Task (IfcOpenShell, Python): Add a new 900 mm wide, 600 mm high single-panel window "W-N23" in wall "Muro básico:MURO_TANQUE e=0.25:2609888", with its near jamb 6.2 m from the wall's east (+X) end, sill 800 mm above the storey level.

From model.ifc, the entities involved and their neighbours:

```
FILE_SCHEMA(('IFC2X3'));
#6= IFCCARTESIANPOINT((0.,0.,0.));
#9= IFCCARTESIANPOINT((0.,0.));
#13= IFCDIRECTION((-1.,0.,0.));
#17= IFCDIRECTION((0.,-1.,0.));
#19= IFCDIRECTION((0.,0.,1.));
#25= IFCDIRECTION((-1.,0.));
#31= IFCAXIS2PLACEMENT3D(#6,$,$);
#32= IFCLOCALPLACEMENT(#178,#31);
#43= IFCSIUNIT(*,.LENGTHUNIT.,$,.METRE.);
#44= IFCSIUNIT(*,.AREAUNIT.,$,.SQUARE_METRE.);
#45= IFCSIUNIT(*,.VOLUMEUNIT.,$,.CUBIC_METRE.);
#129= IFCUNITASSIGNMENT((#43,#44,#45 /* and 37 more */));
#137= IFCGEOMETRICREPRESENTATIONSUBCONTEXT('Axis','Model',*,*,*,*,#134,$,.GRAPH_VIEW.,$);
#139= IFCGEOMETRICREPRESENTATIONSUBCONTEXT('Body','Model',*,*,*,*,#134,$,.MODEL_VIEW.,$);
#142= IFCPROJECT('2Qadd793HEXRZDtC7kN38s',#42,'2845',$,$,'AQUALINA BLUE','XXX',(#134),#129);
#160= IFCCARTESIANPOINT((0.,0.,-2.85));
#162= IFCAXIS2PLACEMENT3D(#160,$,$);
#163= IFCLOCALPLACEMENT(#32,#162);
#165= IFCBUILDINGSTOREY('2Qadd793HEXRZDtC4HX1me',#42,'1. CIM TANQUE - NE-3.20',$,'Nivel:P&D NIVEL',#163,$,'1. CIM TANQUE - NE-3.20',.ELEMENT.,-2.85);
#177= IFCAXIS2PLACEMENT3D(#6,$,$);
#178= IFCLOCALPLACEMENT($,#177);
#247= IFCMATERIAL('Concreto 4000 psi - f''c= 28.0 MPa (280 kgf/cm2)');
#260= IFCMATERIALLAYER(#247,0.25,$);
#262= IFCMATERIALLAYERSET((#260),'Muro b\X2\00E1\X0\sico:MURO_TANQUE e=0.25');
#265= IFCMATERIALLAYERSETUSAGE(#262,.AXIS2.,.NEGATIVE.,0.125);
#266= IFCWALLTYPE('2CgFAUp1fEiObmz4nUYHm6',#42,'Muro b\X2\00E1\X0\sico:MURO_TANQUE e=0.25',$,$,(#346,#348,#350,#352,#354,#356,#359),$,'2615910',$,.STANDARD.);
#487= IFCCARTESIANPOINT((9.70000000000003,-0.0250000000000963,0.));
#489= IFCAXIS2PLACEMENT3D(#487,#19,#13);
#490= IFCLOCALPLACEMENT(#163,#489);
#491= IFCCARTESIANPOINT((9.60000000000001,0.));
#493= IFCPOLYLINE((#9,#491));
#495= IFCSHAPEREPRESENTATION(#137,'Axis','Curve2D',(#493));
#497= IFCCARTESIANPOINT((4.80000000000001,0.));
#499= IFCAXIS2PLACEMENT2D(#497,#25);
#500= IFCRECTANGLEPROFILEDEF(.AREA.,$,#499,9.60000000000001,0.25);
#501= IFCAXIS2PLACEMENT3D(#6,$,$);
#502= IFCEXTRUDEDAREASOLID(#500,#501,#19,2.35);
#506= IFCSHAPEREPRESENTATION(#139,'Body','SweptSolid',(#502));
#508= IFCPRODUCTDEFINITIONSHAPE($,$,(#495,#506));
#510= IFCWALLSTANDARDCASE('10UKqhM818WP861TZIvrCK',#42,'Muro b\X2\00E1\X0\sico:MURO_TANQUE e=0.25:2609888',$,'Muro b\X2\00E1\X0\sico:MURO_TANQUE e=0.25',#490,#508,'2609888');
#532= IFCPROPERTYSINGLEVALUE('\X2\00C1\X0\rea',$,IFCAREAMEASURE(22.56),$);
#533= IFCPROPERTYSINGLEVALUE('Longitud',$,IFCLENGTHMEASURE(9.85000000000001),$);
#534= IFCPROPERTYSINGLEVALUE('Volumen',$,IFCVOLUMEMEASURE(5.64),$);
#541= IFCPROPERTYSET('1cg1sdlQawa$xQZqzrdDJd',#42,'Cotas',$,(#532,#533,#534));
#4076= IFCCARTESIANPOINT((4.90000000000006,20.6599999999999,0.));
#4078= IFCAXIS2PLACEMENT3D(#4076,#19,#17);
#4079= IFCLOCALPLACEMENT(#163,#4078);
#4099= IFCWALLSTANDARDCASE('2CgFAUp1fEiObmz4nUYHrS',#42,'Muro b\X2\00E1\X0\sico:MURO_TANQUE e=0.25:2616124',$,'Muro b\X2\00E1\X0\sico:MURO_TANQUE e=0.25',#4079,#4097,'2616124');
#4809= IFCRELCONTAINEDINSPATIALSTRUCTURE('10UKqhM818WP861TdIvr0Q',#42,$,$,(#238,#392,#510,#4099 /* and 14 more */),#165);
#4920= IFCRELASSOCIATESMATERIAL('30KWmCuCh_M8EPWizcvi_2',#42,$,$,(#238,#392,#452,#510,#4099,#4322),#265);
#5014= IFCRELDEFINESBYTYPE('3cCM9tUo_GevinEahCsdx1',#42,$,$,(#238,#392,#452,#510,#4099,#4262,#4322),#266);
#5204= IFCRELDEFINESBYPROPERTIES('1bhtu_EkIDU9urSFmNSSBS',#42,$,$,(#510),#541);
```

```python
import numpy as np
import ifcopenshell
import ifcopenshell.api.feature
import ifcopenshell.api.geometry
import ifcopenshell.api.pset
import ifcopenshell.api.root
import ifcopenshell.api.spatial
import ifcopenshell.api.type
import ifcopenshell.geom
import ifcopenshell.util.element
import ifcopenshell.util.placement
import ifcopenshell.util.representation
import ifcopenshell.util.shape
import ifcopenshell.util.unit

model = ifcopenshell.open("model.ifc")
unit_scale = ifcopenshell.util.unit.calculate_unit_scale(model)
area_scale = ifcopenshell.util.unit.calculate_unit_scale(model, "AREAUNIT")
volume_scale = ifcopenshell.util.unit.calculate_unit_scale(model, "VOLUMEUNIT")
settings = ifcopenshell.geom.settings()


def volume(element):
    """Net volume in cubic metres, openings subtracted."""
    shape = ifcopenshell.geom.create_shape(settings, element)
    return ifcopenshell.util.shape.get_volume(shape.geometry)


wall = model.by_guid("10UKqhM818WP861TZIvrCK")
storey = ifcopenshell.util.element.get_container(wall, ifc_class="IfcBuildingStorey")
context = ifcopenshell.util.representation.get_context(model, "Model", "Body", "MODEL_VIEW")
before = volume(wall)

width, height, from_end, sill = 0.9, 0.6, 6.2, 0.8  # metres

# The wall runs along its own X axis, and the end named is its -X end.
wall_shape = ifcopenshell.geom.create_shape(settings, wall)
x, y, z = ifcopenshell.util.shape.get_vertices(wall_shape.geometry).T
start = x.min() + from_end
face, thickness = float(y.min()), float(y.max() - y.min())
wall_matrix = ifcopenshell.util.placement.get_local_placement(wall.ObjectPlacement)
level = ifcopenshell.util.placement.get_local_placement(storey.ObjectPlacement)[2, 3]


def in_wall(x, y):
    """Placement at x, y metres in the wall's axes, at sill height."""
    matrix = wall_matrix.copy()
    matrix[:, 3] = wall_matrix @ np.array([x / unit_scale, y / unit_scale, 0.0, 1.0])
    matrix[2, 3] = level + sill / unit_scale
    return matrix


# Opening: a box that overshoots both wall faces by 50 mm.
opening = ifcopenshell.api.root.create_entity(model, ifc_class="IfcOpeningElement")
box = ifcopenshell.api.geometry.add_wall_representation(
    model, context=context, length=width, height=height, thickness=thickness + 0.1
)
ifcopenshell.api.geometry.assign_representation(model, product=opening, representation=box)
ifcopenshell.api.geometry.edit_object_placement(model, product=opening, matrix=in_wall(start, face - 0.05), is_si=False)
ifcopenshell.api.feature.add_feature(model, feature=opening, element=wall)

window = ifcopenshell.api.root.create_entity(model, ifc_class="IfcWindow", name="W-N23")
window.OverallWidth, window.OverallHeight = width / unit_scale, height / unit_scale
body = ifcopenshell.api.geometry.add_window_representation(
    model,
    context=context,
    overall_width=window.OverallWidth,
    overall_height=window.OverallHeight,
    partition_type="SINGLE_PANEL",
)
ifcopenshell.api.geometry.assign_representation(model, product=window, representation=body)
ifcopenshell.api.spatial.assign_container(model, products=[window], relating_structure=storey)
fills = ifcopenshell.api.feature.add_filling(model, opening=opening, element=window)
fills.OwnerHistory = window.OwnerHistory  # required in IFC2X3

# IFC2X3 keeps the operation on the window style.
style = ifcopenshell.api.root.create_entity(model, ifc_class="IfcWindowStyle", name="W-N23")
style.OperationType, style.ConstructionType = "SINGLE_PANEL", "NOTDEFINED"
style.ParameterTakesPrecedence = style.Sizeable = False
ifcopenshell.api.type.assign_type(model, related_objects=[window], relating_type=style)

# Centre the window in the wall's thickness.
ifcopenshell.api.geometry.edit_object_placement(model, product=window, matrix=in_wall(start, face), is_si=False)
window_shape = ifcopenshell.geom.create_shape(settings, window)
depth = ifcopenshell.util.shape.get_vertices(window_shape.geometry)[:, 1]
offset = face + thickness / 2 - (depth.min() + depth.max()) / 2
ifcopenshell.api.geometry.edit_object_placement(model, product=window, matrix=in_wall(start, offset), is_si=False)

after = volume(wall)

# Update the wall's stored quantities.
pset = model.by_id(ifcopenshell.util.element.get_pset(wall, "Cotas", should_inherit=False)["id"])
ifcopenshell.api.pset.edit_pset(model, pset=pset, properties={
    "Área": model.create_entity("IfcAreaMeasure", after / thickness / area_scale),
    "Volumen": model.create_entity("IfcVolumeMeasure", after / volume_scale),
})

print(f"wall volume {before:.3f} -> {after:.3f} m3")

model.write("model_rev.ifc")
```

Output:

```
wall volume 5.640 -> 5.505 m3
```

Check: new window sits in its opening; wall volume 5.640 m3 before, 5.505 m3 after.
